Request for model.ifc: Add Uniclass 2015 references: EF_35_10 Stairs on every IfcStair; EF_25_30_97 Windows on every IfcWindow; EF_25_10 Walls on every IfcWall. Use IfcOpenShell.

First a look at what the model holds.

```python
import ifcopenshell

model = ifcopenshell.open("model.ifc")
print(model.schema)
print("classifications:", [c.Name for c in model.by_type("IfcClassification")])
for ifc_class in ("IfcDoor", "IfcRoof", "IfcStair", "IfcWall", "IfcWindow"):
    print(ifc_class, len(model.by_type(ifc_class)))
```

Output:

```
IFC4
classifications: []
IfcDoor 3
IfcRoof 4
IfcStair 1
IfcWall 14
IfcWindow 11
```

```python
import ifcopenshell
import ifcopenshell.api.classification

model = ifcopenshell.open("model.ifc")

system = ifcopenshell.api.classification.add_classification(model, classification="Uniclass 2015")

codes = {
    "IfcStair": ("EF_35_10", "Stairs"),
    "IfcWindow": ("EF_25_30_97", "Windows"),
    "IfcWall": ("EF_25_10", "Walls"),
}
for ifc_class, (code, name) in codes.items():
    products = model.by_type(ifc_class)
    ifcopenshell.api.classification.add_reference(
        model, products=products, classification=system, identification=code, name=name
    )
    print(code, len(products))

model.write("model_edited.ifc")
```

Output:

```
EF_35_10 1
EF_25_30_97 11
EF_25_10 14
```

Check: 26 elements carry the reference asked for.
